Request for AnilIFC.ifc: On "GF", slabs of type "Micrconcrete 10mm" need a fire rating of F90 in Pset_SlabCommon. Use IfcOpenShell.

First a look at what the model holds.

```python
import ifcopenshell
import ifcopenshell.util.element

model = ifcopenshell.open("AnilIFC.ifc")
print(model.schema)
storey = next(s for s in model.by_type("IfcBuildingStorey") if s.Name == "GF")
slabs = [e for e in ifcopenshell.util.element.get_decomposition(storey) if e.is_a("IfcSlab")]
seen = {}
for e in slabs:
    element_type = ifcopenshell.util.element.get_type(e)
    key = (element_type.Name if element_type != e and element_type else None, ifcopenshell.util.element.get_pset(e, "Pset_SlabCommon", "FireRating"))
    seen[key] = seen.get(key, 0) + 1
for (name, value), count in sorted(seen.items(), key=str):
    print(count, "x", name, "|", value)
```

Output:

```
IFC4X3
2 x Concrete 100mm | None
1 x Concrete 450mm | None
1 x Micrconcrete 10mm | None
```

```python
import ifcopenshell
import ifcopenshell.api.pset
import ifcopenshell.util.element

model = ifcopenshell.open("AnilIFC.ifc")

storey = next(s for s in model.by_type("IfcBuildingStorey") if s.Name == "GF")
slabs = [e for e in ifcopenshell.util.element.get_decomposition(storey) if e.is_a("IfcSlab")]

count = 0
for e in slabs:
    element_type = ifcopenshell.util.element.get_type(e)
    if element_type in (None, e) or element_type.Name != "Micrconcrete 10mm":
        continue
    # add_pset returns the element's existing set when there is one.
    pset = ifcopenshell.api.pset.add_pset(model, product=e, name="Pset_SlabCommon")
    ifcopenshell.api.pset.edit_pset(model, pset=pset, properties={"FireRating": "F90"})
    count += 1

print(count, "slabs updated")

model.write("AnilIFC-out.ifc")
```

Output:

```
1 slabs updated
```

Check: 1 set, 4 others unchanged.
